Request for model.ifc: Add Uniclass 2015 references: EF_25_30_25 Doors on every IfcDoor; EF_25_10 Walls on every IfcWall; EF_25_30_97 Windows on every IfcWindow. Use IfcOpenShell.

First a look at what the model holds.

```python
import ifcopenshell

model = ifcopenshell.open("model.ifc")
print(model.schema)
print("classifications:", [c.Name for c in model.by_type("IfcClassification")])
for ifc_class in ("IfcDoor", "IfcRoof", "IfcStair", "IfcWall", "IfcWindow"):
    print(ifc_class, len(model.by_type(ifc_class)))
```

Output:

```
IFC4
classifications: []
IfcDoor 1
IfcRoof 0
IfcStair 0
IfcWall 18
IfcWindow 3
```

```python
import ifcopenshell
import ifcopenshell.api.classification

model = ifcopenshell.open("model.ifc")

system = ifcopenshell.api.classification.add_classification(model, classification="Uniclass 2015")

codes = {
    "IfcDoor": ("EF_25_30_25", "Doors"),
    "IfcWall": ("EF_25_10", "Walls"),
    "IfcWindow": ("EF_25_30_97", "Windows"),
}
for ifc_class, (code, name) in codes.items():
    products = model.by_type(ifc_class)
    ifcopenshell.api.classification.add_reference(
        model, products=products, classification=system, identification=code, name=name
    )
    print(code, len(products))

model.write("model_v2.ifc")
```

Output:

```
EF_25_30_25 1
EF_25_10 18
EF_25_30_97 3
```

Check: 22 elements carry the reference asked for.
